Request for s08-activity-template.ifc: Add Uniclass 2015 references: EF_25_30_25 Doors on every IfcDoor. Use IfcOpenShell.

First a look at what the model holds.

```python
import ifcopenshell

model = ifcopenshell.open("s08-activity-template.ifc")
print(model.schema)
print("classifications:", [c.Name for c in model.by_type("IfcClassification")])
for ifc_class in ("IfcDoor", "IfcRoof", "IfcStair", "IfcWall", "IfcWindow"):
    print(ifc_class, len(model.by_type(ifc_class)))
```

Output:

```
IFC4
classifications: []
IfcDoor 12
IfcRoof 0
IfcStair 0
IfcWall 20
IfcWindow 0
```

```python
import ifcopenshell
import ifcopenshell.api.classification

model = ifcopenshell.open("s08-activity-template.ifc")

system = ifcopenshell.api.classification.add_classification(model, classification="Uniclass 2015")

codes = {
    "IfcDoor": ("EF_25_30_25", "Doors"),
}
for ifc_class, (code, name) in codes.items():
    products = model.by_type(ifc_class)
    ifcopenshell.api.classification.add_reference(
        model, products=products, classification=system, identification=code, name=name
    )
    print(code, len(products))

model.write("s08-activity-template-out.ifc")
```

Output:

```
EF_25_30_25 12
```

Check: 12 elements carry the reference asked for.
